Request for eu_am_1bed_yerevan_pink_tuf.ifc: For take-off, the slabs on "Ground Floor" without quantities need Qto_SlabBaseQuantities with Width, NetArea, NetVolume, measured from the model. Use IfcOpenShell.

First a look at what the model holds.

```python
import ifcopenshell
import ifcopenshell.util.element
import ifcopenshell.util.unit

model = ifcopenshell.open("eu_am_1bed_yerevan_pink_tuf.ifc")
print(model.schema)
for unit_type in ("LENGTHUNIT", "AREAUNIT", "VOLUMEUNIT"):
    print(unit_type, ifcopenshell.util.unit.calculate_unit_scale(model, unit_type))
storey = next(s for s in model.by_type("IfcBuildingStorey") if s.Name == "Ground Floor")
slabs = [e for e in ifcopenshell.util.element.get_decomposition(storey) if e.is_a("IfcSlab")]
for e in sorted(slabs, key=lambda e: e.id()):
    print(e.id(), e.is_a(), e.Name, list(ifcopenshell.util.element.get_psets(e, qtos_only=True)), sep=" | ")
```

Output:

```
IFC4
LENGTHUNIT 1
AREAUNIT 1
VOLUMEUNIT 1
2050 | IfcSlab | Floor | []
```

```python
import ifcopenshell
import ifcopenshell.api.pset
import ifcopenshell.geom
import ifcopenshell.util.element
import ifcopenshell.util.shape
import ifcopenshell.util.unit

model = ifcopenshell.open("eu_am_1bed_yerevan_pink_tuf.ifc")
unit_scale = ifcopenshell.util.unit.calculate_unit_scale(model)
area_scale = ifcopenshell.util.unit.calculate_unit_scale(model, "AREAUNIT")
volume_scale = ifcopenshell.util.unit.calculate_unit_scale(model, "VOLUMEUNIT")
settings = ifcopenshell.geom.settings()

storey = next(s for s in model.by_type("IfcBuildingStorey") if s.Name == "Ground Floor")
slabs = [e for e in ifcopenshell.util.element.get_decomposition(storey) if e.is_a("IfcSlab")]

for e in sorted(slabs, key=lambda e: e.id()):
    if ifcopenshell.util.element.get_psets(e, qtos_only=True, should_inherit=False):
        continue
    # Geometry comes back in metres, in the element's own axes.
    shape = ifcopenshell.geom.create_shape(settings, e)
    values = {
        "Width": ifcopenshell.util.shape.get_z(shape.geometry) / unit_scale,
        "NetArea": ifcopenshell.util.shape.get_footprint_area(shape.geometry) / area_scale,
        "NetVolume": ifcopenshell.util.shape.get_volume(shape.geometry) / volume_scale,
    }
    qto = ifcopenshell.api.pset.add_qto(model, product=e, name="Qto_SlabBaseQuantities")
    ifcopenshell.api.pset.edit_qto(model, qto=qto, properties=values)
    print(e.id(), {k: round(v, 3) for k, v in values.items()})

model.write("eu_am_1bed_yerevan_pink_tuf_rev.ifc")
```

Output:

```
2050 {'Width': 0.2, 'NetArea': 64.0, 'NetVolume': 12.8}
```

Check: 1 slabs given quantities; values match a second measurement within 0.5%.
